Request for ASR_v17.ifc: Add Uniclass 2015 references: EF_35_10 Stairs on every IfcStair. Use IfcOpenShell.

First a look at what the model holds.

```python
import ifcopenshell

model = ifcopenshell.open("ASR_v17.ifc")
print(model.schema)
print("classifications:", [c.Name for c in model.by_type("IfcClassification")])
for ifc_class in ("IfcDoor", "IfcRoof", "IfcStair", "IfcWall", "IfcWindow"):
    print(ifc_class, len(model.by_type(ifc_class)))
```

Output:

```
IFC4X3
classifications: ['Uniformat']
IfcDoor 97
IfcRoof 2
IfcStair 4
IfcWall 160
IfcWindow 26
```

```python
import ifcopenshell
import ifcopenshell.api.classification

model = ifcopenshell.open("ASR_v17.ifc")

system = ifcopenshell.api.classification.add_classification(model, classification="Uniclass 2015")

codes = {
    "IfcStair": ("EF_35_10", "Stairs"),
}
for ifc_class, (code, name) in codes.items():
    products = model.by_type(ifc_class)
    ifcopenshell.api.classification.add_reference(
        model, products=products, classification=system, identification=code, name=name
    )
    print(code, len(products))

model.write("ASR_v17-out.ifc")
```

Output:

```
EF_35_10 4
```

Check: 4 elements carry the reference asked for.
